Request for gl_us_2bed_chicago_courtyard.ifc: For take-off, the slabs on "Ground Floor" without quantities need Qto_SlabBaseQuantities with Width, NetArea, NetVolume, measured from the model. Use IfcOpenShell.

First a look at what the model holds.

```python
import ifcopenshell
import ifcopenshell.util.element
import ifcopenshell.util.unit

model = ifcopenshell.open("gl_us_2bed_chicago_courtyard.ifc")
print(model.schema)
for unit_type in ("LENGTHUNIT", "AREAUNIT", "VOLUMEUNIT"):
    print(unit_type, ifcopenshell.util.unit.calculate_unit_scale(model, unit_type))
storey = next(s for s in model.by_type("IfcBuildingStorey") if s.Name == "Ground Floor")
slabs = [e for e in ifcopenshell.util.element.get_decomposition(storey) if e.is_a("IfcSlab")]
for e in sorted(slabs, key=lambda e: e.id()):
    print(e.id(), e.is_a(), e.Name, list(ifcopenshell.util.element.get_psets(e, qtos_only=True)), sep=" | ")
```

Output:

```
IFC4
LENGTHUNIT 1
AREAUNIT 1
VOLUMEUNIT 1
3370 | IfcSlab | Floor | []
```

```python
import ifcopenshell
import ifcopenshell.api.pset
import ifcopenshell.geom
import ifcopenshell.util.element
import ifcopenshell.util.shape
import ifcopenshell.util.unit

model = ifcopenshell.open("gl_us_2bed_chicago_courtyard.ifc")
unit_scale = ifcopenshell.util.unit.calculate_unit_scale(model)
area_scale = ifcopenshell.util.unit.calculate_unit_scale(model, "AREAUNIT")
volume_scale = ifcopenshell.util.unit.calculate_unit_scale(model, "VOLUMEUNIT")
settings = ifcopenshell.geom.settings()

storey = next(s for s in model.by_type("IfcBuildingStorey") if s.Name == "Ground Floor")
slabs = [e for e in ifcopenshell.util.element.get_decomposition(storey) if e.is_a("IfcSlab")]

for e in sorted(slabs, key=lambda e: e.id()):
    if ifcopenshell.util.element.get_psets(e, qtos_only=True, should_inherit=False):
        continue
    # Geometry comes back in metres, in the element's own axes.
    shape = ifcopenshell.geom.create_shape(settings, e)
    values = {
        "Width": ifcopenshell.util.shape.get_z(shape.geometry) / unit_scale,
        "NetArea": ifcopenshell.util.shape.get_footprint_area(shape.geometry) / area_scale,
        "NetVolume": ifcopenshell.util.shape.get_volume(shape.geometry) / volume_scale,
    }
    qto = ifcopenshell.api.pset.add_qto(model, product=e, name="Qto_SlabBaseQuantities")
    ifcopenshell.api.pset.edit_qto(model, qto=qto, properties=values)
    print(e.id(), {k: round(v, 3) for k, v in values.items()})

model.write("gl_us_2bed_chicago_courtyard-out.ifc")
```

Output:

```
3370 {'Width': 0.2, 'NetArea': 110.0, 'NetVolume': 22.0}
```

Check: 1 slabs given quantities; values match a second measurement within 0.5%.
